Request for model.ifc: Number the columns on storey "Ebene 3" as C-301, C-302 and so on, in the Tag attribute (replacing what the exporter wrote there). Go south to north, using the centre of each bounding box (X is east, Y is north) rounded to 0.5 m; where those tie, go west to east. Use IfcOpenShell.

First a look at what the model holds.

```python
import ifcopenshell
import ifcopenshell.util.element
import ifcopenshell.util.placement

model = ifcopenshell.open("model.ifc")
print(model.schema)
storey = next(s for s in model.by_type("IfcBuildingStorey") if s.Name == "Ebene 3")
columns = [e for e in ifcopenshell.util.element.get_decomposition(storey) if e.is_a("IfcColumn")]
for e in sorted(columns, key=lambda e: e.id()):
    origin = ifcopenshell.util.placement.get_local_placement(e.ObjectPlacement)[:3, 3]
    print(e.id(), e.Tag, e.Name, origin.round(2) + 0.0, sep=" | ")
```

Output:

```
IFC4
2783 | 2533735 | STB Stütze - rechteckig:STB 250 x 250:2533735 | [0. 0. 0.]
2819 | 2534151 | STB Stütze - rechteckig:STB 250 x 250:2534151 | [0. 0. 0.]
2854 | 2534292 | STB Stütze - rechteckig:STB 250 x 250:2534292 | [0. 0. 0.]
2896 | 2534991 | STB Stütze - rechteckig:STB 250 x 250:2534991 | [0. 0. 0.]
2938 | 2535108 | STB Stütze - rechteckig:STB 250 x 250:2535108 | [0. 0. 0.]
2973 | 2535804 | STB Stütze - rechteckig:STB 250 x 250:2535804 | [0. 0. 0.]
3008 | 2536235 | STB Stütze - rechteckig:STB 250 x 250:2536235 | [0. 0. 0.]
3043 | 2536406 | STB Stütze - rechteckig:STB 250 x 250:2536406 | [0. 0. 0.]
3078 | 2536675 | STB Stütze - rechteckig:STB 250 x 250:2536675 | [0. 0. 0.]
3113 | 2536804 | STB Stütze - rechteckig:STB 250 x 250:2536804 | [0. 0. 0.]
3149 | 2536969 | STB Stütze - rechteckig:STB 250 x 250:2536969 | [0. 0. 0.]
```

```python
import ifcopenshell
import ifcopenshell.geom
import ifcopenshell.util.element
import ifcopenshell.util.shape

model = ifcopenshell.open("model.ifc")
settings = ifcopenshell.geom.settings()
settings.set("use-world-coords", True)


def centre(element):
    shape = ifcopenshell.geom.create_shape(settings, element)
    return ifcopenshell.util.shape.get_bbox_centroid(shape.geometry)


storey = next(s for s in model.by_type("IfcBuildingStorey") if s.Name == "Ebene 3")
columns = [e for e in ifcopenshell.util.element.get_decomposition(storey) if e.is_a("IfcColumn")]

# Insertion points can sit at a corner or the storey origin, so sort by the geometry (in metres).
centres = {e: centre(e) for e in columns}
columns.sort(key=lambda e: (round(centres[e][1] / 0.5), centres[e][0]))

for i, e in enumerate(columns, start=1):
    number = f"C-3{i:02d}"
    e.Tag = number
    print(e.id(), number)

model.write("model-out.ifc")
```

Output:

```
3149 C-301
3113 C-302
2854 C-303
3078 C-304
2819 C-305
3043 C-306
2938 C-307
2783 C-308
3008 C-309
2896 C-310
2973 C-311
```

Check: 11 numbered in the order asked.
